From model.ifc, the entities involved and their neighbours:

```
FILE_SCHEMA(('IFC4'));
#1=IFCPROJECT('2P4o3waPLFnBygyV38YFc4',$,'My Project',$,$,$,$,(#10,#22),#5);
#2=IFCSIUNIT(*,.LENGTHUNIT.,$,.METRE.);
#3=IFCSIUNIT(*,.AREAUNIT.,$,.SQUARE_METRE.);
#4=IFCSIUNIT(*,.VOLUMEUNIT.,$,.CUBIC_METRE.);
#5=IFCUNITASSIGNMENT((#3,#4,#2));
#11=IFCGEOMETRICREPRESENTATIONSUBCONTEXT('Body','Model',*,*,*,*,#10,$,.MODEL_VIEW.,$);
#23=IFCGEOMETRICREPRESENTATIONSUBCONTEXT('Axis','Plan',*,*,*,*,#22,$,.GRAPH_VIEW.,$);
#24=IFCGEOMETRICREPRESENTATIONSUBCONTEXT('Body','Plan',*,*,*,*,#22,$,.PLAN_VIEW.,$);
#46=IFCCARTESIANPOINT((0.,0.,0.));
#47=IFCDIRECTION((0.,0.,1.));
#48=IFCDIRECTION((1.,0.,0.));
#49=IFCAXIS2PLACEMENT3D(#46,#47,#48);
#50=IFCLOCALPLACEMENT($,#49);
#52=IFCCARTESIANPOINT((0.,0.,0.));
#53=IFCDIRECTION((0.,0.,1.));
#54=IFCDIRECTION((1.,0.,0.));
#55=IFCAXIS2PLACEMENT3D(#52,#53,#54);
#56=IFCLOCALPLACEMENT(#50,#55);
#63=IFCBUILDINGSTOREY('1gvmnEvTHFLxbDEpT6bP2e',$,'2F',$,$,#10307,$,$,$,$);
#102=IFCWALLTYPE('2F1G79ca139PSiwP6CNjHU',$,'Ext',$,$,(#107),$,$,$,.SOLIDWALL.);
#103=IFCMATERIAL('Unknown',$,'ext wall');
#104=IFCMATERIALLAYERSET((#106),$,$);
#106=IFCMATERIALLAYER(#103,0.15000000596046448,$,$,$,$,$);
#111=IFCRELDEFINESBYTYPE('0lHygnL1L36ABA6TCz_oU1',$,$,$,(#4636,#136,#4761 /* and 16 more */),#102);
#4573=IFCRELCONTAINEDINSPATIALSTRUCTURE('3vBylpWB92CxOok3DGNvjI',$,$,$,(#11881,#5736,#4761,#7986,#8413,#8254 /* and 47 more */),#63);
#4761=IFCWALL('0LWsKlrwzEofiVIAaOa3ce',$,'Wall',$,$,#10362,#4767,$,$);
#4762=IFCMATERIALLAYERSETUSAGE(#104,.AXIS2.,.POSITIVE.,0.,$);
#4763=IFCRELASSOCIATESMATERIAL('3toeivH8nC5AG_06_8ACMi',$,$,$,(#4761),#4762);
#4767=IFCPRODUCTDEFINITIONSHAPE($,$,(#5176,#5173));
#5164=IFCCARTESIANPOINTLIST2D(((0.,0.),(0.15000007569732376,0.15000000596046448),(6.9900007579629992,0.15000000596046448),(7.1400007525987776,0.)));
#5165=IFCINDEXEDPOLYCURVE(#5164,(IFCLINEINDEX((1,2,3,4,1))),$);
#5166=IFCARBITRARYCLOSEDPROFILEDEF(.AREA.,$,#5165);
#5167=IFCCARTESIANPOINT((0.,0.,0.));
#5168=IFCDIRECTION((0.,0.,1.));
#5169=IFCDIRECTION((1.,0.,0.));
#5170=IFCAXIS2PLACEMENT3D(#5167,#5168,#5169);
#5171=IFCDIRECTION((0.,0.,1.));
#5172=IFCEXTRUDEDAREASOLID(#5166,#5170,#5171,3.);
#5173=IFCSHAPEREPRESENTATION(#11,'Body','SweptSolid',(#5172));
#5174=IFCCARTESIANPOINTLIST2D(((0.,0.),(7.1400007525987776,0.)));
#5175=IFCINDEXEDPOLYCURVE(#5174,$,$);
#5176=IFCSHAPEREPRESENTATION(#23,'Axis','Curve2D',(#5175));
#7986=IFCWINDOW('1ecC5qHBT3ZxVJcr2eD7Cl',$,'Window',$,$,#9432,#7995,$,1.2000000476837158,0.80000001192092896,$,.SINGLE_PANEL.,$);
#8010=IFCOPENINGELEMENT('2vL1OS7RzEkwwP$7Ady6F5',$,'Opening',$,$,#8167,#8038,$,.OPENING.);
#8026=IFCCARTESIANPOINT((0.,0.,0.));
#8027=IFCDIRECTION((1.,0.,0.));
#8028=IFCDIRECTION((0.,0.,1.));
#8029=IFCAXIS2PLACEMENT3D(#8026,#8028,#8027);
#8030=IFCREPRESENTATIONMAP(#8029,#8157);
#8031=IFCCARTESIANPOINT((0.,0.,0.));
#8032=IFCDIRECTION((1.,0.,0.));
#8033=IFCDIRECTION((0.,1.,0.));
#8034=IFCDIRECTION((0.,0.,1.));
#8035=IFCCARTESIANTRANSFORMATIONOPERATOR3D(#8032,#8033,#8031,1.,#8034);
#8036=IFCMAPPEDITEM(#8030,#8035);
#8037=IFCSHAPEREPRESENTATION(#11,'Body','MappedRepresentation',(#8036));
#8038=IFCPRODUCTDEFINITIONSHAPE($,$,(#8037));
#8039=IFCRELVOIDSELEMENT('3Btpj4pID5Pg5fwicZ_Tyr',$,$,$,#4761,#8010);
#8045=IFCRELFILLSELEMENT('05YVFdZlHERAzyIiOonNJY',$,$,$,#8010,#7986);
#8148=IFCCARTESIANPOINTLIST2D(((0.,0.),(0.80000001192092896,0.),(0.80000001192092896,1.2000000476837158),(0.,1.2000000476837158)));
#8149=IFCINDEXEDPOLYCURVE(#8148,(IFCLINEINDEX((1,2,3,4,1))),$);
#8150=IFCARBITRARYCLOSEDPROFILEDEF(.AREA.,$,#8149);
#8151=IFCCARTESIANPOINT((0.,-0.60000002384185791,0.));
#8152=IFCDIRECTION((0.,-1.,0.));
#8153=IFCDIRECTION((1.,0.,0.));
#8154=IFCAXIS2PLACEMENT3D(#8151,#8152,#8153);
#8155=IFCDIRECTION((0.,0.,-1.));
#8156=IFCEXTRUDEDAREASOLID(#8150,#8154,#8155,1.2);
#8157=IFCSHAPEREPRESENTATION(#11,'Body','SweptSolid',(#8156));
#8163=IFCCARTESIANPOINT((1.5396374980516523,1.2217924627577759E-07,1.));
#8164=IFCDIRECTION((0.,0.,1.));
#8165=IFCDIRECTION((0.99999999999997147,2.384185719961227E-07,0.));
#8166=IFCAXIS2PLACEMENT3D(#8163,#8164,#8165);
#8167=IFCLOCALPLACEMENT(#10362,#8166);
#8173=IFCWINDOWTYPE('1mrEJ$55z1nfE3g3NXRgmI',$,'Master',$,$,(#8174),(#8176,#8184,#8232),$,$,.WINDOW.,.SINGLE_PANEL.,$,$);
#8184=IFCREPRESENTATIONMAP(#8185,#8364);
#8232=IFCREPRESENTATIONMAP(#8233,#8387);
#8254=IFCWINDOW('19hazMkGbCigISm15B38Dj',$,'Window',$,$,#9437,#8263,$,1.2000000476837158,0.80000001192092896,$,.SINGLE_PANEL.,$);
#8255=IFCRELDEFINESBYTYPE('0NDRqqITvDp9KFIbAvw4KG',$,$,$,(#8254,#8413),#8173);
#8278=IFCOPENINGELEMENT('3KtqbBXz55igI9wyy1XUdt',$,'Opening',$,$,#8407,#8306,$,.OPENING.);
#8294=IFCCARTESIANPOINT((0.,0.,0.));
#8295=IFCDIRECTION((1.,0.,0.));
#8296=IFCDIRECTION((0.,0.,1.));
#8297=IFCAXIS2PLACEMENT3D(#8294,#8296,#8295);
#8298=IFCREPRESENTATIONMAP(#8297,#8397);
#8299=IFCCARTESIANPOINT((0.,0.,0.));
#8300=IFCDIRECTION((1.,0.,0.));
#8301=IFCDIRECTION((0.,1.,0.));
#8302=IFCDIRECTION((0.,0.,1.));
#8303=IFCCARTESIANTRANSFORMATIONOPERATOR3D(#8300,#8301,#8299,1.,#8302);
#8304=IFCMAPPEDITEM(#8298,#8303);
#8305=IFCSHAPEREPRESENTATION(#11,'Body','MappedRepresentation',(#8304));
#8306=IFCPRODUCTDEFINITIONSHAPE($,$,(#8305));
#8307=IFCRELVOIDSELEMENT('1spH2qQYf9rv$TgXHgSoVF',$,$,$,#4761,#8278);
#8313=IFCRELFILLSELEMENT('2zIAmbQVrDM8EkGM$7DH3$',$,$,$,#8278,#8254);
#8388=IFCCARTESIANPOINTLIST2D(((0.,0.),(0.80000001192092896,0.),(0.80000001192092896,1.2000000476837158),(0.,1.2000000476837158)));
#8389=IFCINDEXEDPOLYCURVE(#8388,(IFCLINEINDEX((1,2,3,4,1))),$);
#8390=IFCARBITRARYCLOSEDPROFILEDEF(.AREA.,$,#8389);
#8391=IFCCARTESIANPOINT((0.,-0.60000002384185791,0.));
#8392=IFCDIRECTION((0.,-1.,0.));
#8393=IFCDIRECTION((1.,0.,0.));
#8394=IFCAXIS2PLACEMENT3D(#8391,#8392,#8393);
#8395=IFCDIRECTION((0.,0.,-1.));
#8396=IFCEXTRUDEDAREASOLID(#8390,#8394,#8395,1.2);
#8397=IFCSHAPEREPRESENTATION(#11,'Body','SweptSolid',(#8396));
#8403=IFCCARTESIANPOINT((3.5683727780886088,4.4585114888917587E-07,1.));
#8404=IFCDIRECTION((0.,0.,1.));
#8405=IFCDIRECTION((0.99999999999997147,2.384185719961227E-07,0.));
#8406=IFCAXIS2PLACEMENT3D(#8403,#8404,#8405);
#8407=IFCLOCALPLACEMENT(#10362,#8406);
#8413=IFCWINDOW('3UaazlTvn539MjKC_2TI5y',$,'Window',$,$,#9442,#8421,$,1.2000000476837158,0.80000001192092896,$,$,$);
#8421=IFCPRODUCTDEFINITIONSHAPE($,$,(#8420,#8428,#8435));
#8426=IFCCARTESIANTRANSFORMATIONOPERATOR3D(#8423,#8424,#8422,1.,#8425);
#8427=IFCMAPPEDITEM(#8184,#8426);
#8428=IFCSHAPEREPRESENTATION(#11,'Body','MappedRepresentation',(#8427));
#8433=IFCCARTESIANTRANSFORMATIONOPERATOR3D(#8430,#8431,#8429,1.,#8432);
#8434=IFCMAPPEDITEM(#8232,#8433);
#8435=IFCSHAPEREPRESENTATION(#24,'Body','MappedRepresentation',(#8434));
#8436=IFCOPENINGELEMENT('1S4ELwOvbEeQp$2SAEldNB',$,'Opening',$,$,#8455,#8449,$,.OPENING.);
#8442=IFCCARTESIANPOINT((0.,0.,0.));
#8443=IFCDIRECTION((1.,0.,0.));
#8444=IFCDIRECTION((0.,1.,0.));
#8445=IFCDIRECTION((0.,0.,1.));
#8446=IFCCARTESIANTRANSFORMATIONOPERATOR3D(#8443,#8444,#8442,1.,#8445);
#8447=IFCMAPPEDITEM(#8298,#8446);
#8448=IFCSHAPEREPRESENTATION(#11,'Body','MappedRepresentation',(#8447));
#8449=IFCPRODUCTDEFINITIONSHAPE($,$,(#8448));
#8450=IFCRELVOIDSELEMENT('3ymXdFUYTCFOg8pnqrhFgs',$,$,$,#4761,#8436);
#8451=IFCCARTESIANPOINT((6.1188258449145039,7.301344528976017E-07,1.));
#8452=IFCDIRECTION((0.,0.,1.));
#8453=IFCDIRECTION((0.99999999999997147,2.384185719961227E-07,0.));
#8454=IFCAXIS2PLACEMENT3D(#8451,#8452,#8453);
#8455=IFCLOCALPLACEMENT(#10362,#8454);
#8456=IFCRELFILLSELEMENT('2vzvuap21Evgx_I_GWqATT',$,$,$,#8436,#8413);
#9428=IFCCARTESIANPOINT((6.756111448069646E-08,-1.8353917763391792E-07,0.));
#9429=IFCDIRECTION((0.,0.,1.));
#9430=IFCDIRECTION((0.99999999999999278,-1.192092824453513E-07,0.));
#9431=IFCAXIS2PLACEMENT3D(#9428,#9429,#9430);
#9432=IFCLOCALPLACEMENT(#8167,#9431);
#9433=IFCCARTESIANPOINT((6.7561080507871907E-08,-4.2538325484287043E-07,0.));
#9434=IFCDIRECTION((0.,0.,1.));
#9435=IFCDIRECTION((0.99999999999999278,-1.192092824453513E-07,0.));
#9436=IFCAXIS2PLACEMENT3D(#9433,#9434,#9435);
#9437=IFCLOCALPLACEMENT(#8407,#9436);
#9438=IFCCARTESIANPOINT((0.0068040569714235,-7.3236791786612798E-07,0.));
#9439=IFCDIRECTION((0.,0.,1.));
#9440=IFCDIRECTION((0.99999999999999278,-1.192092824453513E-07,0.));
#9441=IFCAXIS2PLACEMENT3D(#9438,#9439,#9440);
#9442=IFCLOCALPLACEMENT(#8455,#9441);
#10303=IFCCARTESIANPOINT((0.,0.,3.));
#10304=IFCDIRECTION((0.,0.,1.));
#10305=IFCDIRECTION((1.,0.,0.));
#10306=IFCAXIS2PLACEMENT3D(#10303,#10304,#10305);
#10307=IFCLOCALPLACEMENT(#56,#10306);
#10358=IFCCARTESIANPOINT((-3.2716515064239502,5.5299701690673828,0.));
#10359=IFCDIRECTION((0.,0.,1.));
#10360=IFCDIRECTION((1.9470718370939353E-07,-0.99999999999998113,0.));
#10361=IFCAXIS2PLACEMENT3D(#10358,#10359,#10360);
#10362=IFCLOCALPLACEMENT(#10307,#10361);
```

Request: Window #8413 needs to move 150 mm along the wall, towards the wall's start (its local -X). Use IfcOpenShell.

```python
import ifcopenshell
import ifcopenshell.api.geometry
import ifcopenshell.util.placement
import ifcopenshell.util.unit

model = ifcopenshell.open("model.ifc")
unit_scale = ifcopenshell.util.unit.calculate_unit_scale(model)

window = model.by_guid("3UaazlTvn539MjKC_2TI5y")
opening = window.FillsVoids[0].RelatingOpeningElement
wall = opening.VoidsElements[0].RelatingBuildingElement

wall_matrix = ifcopenshell.util.placement.get_local_placement(wall.ObjectPlacement)
shift = wall_matrix[:3, 0] * -0.15 / unit_scale
before = ifcopenshell.util.placement.get_local_placement(window.ObjectPlacement)[:3, 3].copy()

# The window is placed relative to its opening, so it follows when the opening moves.
matrix = ifcopenshell.util.placement.get_local_placement(opening.ObjectPlacement)
matrix[:3, 3] += shift
ifcopenshell.api.geometry.edit_object_placement(
    model, product=opening, matrix=matrix, is_si=False, should_transform_children=True
)

after = ifcopenshell.util.placement.get_local_placement(window.ObjectPlacement)[:3, 3]
print("window moved by", (after - before).round(3) + 0.0)

model.write("model_rev.ifc")
```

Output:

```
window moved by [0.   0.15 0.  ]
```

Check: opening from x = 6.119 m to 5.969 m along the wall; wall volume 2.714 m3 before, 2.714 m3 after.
